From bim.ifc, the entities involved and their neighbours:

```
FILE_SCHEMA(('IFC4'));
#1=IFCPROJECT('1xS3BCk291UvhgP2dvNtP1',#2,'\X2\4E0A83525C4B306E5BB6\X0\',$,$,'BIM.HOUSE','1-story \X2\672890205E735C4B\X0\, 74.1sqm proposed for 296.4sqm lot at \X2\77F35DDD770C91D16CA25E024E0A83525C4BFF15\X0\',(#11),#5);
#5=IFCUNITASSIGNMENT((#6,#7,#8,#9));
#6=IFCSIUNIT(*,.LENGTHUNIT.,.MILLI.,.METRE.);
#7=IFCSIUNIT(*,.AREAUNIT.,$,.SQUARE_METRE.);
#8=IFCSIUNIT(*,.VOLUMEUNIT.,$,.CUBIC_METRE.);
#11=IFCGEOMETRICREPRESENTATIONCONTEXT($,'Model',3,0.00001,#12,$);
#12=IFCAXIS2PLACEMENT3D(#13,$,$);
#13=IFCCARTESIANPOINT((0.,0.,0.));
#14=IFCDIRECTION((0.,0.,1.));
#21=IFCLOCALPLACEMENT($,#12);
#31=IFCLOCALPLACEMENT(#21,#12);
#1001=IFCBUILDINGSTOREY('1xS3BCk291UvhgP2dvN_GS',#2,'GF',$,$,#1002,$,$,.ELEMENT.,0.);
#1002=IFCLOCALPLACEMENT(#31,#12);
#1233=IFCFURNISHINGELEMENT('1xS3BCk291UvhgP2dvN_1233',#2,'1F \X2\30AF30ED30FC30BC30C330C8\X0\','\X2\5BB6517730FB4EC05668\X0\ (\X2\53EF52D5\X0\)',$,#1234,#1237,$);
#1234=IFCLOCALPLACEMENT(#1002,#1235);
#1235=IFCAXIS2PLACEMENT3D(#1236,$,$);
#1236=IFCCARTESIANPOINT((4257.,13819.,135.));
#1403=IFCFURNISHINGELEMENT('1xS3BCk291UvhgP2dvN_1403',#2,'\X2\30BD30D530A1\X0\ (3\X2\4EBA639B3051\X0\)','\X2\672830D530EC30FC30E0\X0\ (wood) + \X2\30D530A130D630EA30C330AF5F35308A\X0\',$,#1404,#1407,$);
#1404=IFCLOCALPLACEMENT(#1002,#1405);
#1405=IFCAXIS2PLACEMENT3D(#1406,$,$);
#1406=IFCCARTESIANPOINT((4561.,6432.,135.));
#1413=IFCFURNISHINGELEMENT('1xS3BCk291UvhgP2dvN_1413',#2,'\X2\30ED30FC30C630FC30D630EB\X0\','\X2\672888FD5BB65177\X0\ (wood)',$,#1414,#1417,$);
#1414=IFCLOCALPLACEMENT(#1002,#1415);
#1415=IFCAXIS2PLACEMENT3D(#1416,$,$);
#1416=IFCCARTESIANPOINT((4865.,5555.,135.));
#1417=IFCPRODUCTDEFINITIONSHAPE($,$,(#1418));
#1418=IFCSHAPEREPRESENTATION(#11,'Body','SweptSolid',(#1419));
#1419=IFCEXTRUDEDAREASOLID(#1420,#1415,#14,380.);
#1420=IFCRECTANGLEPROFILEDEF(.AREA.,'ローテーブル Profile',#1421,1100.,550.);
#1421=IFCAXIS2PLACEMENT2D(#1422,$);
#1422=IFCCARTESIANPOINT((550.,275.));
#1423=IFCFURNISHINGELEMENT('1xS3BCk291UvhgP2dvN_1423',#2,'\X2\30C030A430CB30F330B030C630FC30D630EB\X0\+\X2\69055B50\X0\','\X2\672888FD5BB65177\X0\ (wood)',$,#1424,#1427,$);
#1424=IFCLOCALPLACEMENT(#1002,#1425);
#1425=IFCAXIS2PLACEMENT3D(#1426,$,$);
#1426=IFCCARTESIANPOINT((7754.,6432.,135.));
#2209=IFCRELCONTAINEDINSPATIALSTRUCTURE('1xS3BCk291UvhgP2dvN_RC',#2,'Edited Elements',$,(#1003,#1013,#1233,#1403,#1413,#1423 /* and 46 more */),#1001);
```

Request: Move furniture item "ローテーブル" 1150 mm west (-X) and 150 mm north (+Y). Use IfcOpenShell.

```python
import ifcopenshell
import ifcopenshell.api.geometry
import ifcopenshell.util.placement
import ifcopenshell.util.unit

model = ifcopenshell.open("bim.ifc")
unit_scale = ifcopenshell.util.unit.calculate_unit_scale(model)

item = model.by_guid("1xS3BCk291UvhgP2dvN_1413")
matrix = ifcopenshell.util.placement.get_local_placement(item.ObjectPlacement)
matrix[0, 3] -= 1.15 / unit_scale
matrix[1, 3] += 0.15 / unit_scale
ifcopenshell.api.geometry.edit_object_placement(model, product=item, matrix=matrix, is_si=False)

print(ifcopenshell.util.placement.get_local_placement(item.ObjectPlacement).round(3) + 0.0)

model.write("bim_rev.ifc")
```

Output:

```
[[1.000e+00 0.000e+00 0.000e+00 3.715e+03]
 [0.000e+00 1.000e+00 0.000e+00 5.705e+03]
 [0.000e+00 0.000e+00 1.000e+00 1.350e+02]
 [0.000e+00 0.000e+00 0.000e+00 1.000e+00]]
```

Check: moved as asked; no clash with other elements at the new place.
